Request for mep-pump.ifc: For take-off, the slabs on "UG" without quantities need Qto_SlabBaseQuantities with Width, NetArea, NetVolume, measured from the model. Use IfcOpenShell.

First a look at what the model holds.

```python
import ifcopenshell
import ifcopenshell.util.element
import ifcopenshell.util.unit

model = ifcopenshell.open("mep-pump.ifc")
print(model.schema)
for unit_type in ("LENGTHUNIT", "AREAUNIT", "VOLUMEUNIT"):
    print(unit_type, ifcopenshell.util.unit.calculate_unit_scale(model, unit_type))
storey = next(s for s in model.by_type("IfcBuildingStorey") if s.Name == "UG")
slabs = [e for e in ifcopenshell.util.element.get_decomposition(storey) if e.is_a("IfcSlab")]
for e in sorted(slabs, key=lambda e: e.id()):
    print(e.id(), e.is_a(), e.Name, list(ifcopenshell.util.element.get_psets(e, qtos_only=True)), sep=" | ")
```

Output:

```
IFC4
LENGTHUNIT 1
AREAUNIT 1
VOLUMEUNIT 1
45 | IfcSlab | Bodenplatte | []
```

```python
import ifcopenshell
import ifcopenshell.api.pset
import ifcopenshell.geom
import ifcopenshell.util.element
import ifcopenshell.util.shape
import ifcopenshell.util.unit

model = ifcopenshell.open("mep-pump.ifc")
unit_scale = ifcopenshell.util.unit.calculate_unit_scale(model)
area_scale = ifcopenshell.util.unit.calculate_unit_scale(model, "AREAUNIT")
volume_scale = ifcopenshell.util.unit.calculate_unit_scale(model, "VOLUMEUNIT")
settings = ifcopenshell.geom.settings()

storey = next(s for s in model.by_type("IfcBuildingStorey") if s.Name == "UG")
slabs = [e for e in ifcopenshell.util.element.get_decomposition(storey) if e.is_a("IfcSlab")]

for e in sorted(slabs, key=lambda e: e.id()):
    if ifcopenshell.util.element.get_psets(e, qtos_only=True, should_inherit=False):
        continue
    # Geometry comes back in metres, in the element's own axes.
    shape = ifcopenshell.geom.create_shape(settings, e)
    values = {
        "Width": ifcopenshell.util.shape.get_z(shape.geometry) / unit_scale,
        "NetArea": ifcopenshell.util.shape.get_footprint_area(shape.geometry) / area_scale,
        "NetVolume": ifcopenshell.util.shape.get_volume(shape.geometry) / volume_scale,
    }
    qto = ifcopenshell.api.pset.add_qto(model, product=e, name="Qto_SlabBaseQuantities")
    ifcopenshell.api.pset.edit_qto(model, qto=qto, properties=values)
    print(e.id(), {k: round(v, 3) for k, v in values.items()})

model.write("mep-pump-out.ifc")
```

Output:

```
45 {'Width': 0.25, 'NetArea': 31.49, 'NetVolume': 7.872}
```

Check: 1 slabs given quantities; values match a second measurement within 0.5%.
